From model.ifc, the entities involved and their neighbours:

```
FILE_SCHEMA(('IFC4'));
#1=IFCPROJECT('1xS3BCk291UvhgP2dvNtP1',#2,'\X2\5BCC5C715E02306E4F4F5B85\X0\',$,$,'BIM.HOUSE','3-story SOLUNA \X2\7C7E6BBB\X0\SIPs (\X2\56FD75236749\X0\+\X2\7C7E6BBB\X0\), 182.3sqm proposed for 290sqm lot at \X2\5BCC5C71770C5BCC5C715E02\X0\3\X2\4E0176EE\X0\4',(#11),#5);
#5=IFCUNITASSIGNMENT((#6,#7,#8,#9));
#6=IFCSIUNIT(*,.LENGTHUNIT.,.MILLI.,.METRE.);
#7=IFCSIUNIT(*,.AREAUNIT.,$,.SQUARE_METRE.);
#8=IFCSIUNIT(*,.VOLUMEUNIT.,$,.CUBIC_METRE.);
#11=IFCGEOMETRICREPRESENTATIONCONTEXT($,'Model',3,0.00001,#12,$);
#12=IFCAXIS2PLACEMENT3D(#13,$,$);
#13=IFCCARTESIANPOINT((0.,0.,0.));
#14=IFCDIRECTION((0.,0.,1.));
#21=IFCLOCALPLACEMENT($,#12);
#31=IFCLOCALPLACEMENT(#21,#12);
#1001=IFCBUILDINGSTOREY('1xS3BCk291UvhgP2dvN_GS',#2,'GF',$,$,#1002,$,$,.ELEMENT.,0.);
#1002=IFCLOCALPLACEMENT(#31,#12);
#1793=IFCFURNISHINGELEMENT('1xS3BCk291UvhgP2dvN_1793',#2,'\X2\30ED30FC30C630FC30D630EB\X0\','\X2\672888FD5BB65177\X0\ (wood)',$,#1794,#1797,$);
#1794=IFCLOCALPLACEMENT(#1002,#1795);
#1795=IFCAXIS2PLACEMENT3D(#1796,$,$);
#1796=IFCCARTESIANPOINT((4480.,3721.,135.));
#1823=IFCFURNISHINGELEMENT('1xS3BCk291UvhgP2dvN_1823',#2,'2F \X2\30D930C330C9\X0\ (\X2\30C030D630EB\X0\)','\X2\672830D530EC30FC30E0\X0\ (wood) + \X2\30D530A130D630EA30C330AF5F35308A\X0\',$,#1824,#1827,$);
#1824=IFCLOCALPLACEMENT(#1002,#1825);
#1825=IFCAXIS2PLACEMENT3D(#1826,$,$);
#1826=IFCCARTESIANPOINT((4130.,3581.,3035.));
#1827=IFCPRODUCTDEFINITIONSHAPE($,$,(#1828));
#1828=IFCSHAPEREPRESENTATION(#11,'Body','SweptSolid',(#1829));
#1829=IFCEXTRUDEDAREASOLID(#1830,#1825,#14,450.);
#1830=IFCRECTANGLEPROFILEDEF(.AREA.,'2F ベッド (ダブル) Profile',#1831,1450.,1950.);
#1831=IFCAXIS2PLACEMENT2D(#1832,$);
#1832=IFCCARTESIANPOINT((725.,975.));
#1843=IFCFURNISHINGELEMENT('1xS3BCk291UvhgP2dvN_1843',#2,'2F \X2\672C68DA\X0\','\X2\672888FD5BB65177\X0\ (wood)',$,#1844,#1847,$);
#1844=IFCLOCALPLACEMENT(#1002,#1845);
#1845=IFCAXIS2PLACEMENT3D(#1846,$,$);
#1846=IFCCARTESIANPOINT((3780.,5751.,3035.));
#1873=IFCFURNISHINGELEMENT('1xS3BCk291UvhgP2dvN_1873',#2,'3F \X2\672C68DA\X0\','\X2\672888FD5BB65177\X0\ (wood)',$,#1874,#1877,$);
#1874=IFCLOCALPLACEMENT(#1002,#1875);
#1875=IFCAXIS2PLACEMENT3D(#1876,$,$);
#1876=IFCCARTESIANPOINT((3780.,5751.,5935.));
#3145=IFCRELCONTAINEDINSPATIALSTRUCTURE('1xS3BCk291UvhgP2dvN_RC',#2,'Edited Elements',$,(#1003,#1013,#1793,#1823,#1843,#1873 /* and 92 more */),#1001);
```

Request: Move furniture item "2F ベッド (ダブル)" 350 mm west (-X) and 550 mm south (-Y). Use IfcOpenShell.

```python
import ifcopenshell
import ifcopenshell.api.geometry
import ifcopenshell.util.placement
import ifcopenshell.util.unit

model = ifcopenshell.open("model.ifc")
unit_scale = ifcopenshell.util.unit.calculate_unit_scale(model)

item = model.by_id(1823)
matrix = ifcopenshell.util.placement.get_local_placement(item.ObjectPlacement)
matrix[0, 3] -= 0.35 / unit_scale
matrix[1, 3] -= 0.55 / unit_scale
ifcopenshell.api.geometry.edit_object_placement(model, product=item, matrix=matrix, is_si=False)

print(ifcopenshell.util.placement.get_local_placement(item.ObjectPlacement).round(3) + 0.0)

model.write("model_v2.ifc")
```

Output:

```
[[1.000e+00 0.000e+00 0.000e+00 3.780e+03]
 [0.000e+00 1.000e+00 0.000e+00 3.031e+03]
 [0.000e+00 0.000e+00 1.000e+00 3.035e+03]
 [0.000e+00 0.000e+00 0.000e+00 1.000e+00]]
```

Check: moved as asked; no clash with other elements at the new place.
